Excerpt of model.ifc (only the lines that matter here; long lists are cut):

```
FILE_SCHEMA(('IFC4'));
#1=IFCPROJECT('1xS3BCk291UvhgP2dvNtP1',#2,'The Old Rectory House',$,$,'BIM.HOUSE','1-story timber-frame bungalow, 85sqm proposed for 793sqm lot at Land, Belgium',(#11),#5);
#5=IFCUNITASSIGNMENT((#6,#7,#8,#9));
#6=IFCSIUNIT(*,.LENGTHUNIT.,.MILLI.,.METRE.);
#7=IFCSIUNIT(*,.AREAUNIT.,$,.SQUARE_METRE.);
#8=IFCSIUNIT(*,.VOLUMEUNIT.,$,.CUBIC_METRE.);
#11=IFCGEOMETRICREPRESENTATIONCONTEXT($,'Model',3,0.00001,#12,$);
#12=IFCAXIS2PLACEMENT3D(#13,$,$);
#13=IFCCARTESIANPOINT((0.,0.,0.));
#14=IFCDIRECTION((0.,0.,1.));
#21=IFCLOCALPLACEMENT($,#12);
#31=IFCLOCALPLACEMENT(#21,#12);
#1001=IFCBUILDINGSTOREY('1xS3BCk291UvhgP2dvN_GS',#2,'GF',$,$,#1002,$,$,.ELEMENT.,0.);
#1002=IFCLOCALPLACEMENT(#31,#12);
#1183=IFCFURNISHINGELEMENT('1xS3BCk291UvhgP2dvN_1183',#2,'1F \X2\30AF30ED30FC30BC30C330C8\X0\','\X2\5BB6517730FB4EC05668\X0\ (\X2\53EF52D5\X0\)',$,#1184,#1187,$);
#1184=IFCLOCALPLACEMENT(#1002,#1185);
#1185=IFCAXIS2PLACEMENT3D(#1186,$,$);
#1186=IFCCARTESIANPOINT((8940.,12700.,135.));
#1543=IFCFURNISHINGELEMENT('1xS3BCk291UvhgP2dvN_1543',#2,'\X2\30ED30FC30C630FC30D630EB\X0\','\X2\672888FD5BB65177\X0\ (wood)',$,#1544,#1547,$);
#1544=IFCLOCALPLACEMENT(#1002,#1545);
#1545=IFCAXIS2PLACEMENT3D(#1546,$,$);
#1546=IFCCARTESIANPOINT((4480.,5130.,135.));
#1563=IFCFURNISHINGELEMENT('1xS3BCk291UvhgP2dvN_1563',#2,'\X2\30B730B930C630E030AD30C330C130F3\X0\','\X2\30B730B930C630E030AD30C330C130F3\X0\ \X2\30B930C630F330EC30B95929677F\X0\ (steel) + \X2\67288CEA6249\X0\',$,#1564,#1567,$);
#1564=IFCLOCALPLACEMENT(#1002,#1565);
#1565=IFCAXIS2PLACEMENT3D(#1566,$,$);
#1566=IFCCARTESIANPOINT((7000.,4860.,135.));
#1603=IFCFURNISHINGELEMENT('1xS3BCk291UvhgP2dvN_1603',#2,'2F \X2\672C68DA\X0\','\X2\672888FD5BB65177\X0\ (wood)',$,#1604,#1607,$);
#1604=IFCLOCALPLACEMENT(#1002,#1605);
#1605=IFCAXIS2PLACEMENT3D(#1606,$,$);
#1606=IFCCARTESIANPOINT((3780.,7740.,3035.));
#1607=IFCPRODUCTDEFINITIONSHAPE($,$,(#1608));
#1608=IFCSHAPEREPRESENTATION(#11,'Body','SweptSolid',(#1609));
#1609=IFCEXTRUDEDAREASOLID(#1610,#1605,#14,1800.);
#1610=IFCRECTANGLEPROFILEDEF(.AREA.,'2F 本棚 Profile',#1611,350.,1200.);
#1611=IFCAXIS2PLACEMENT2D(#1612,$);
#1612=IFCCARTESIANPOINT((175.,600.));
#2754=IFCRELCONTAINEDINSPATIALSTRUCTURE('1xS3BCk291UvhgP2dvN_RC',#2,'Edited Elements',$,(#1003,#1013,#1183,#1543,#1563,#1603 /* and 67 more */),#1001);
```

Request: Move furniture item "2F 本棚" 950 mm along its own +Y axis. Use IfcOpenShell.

```python
import ifcopenshell
import ifcopenshell.api.geometry
import ifcopenshell.util.placement
import ifcopenshell.util.unit

model = ifcopenshell.open("model.ifc")
unit_scale = ifcopenshell.util.unit.calculate_unit_scale(model)

item = model.by_guid("1xS3BCk291UvhgP2dvN_1603")
matrix = ifcopenshell.util.placement.get_local_placement(item.ObjectPlacement)
matrix[:3, 3] += matrix[:3, 1] * 0.95 / unit_scale
ifcopenshell.api.geometry.edit_object_placement(model, product=item, matrix=matrix, is_si=False)

print(ifcopenshell.util.placement.get_local_placement(item.ObjectPlacement).round(3) + 0.0)

model.write("model_v2.ifc")
```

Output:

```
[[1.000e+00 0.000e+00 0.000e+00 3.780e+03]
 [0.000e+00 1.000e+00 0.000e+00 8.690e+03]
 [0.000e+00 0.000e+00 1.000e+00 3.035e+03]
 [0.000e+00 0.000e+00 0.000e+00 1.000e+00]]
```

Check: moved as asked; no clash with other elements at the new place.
